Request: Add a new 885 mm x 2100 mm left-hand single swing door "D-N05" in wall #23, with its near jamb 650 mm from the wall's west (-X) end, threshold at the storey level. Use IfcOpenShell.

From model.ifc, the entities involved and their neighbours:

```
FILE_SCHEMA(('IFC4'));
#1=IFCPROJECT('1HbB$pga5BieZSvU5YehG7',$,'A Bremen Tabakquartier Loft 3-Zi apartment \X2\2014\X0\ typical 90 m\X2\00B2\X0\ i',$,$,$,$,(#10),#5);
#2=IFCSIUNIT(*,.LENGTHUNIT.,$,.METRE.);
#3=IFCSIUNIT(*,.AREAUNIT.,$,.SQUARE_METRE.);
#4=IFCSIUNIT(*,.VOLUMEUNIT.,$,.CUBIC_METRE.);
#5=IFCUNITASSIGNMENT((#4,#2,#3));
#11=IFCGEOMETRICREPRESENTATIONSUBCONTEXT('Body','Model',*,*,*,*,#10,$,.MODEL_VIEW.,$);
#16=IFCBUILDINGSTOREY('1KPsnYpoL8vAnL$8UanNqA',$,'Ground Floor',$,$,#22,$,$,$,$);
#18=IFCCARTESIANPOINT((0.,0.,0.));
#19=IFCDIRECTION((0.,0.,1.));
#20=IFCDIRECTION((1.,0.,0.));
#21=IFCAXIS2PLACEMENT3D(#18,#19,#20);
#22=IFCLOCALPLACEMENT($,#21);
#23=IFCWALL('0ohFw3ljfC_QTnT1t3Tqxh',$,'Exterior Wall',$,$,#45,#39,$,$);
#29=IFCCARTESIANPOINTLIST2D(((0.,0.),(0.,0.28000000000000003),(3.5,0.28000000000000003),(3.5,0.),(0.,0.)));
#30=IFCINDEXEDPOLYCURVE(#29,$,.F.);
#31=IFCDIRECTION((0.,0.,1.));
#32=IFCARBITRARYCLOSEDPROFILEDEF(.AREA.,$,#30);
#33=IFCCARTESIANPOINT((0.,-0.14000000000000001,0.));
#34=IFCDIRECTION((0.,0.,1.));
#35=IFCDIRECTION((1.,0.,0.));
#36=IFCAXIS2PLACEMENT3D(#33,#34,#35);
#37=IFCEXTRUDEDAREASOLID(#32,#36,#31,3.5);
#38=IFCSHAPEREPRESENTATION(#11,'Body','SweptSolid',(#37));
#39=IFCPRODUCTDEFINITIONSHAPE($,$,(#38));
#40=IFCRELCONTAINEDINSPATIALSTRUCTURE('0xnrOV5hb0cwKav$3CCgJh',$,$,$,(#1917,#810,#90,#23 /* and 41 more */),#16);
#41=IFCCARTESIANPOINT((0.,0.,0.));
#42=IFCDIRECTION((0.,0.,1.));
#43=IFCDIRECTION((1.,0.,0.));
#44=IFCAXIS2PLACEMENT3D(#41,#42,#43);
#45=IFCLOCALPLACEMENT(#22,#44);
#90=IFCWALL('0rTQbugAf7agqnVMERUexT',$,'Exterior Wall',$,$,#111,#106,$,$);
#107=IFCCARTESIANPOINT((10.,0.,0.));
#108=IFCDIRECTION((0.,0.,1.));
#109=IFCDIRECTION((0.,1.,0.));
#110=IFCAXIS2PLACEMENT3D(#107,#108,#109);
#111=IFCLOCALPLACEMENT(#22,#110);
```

```python
import numpy as np
import ifcopenshell
import ifcopenshell.api.feature
import ifcopenshell.api.geometry
import ifcopenshell.api.root
import ifcopenshell.api.spatial
import ifcopenshell.geom
import ifcopenshell.util.element
import ifcopenshell.util.placement
import ifcopenshell.util.representation
import ifcopenshell.util.shape
import ifcopenshell.util.unit

model = ifcopenshell.open("model.ifc")
unit_scale = ifcopenshell.util.unit.calculate_unit_scale(model)
settings = ifcopenshell.geom.settings()


def volume(element):
    """Net volume in cubic metres, openings subtracted."""
    shape = ifcopenshell.geom.create_shape(settings, element)
    return ifcopenshell.util.shape.get_volume(shape.geometry)


wall = model.by_guid("0ohFw3ljfC_QTnT1t3Tqxh")
storey = ifcopenshell.util.element.get_container(wall, ifc_class="IfcBuildingStorey")
context = ifcopenshell.util.representation.get_context(model, "Model", "Body", "MODEL_VIEW")
before = volume(wall)

width, height, from_end, sill = 0.885, 2.1, 0.65, 0.0  # metres

# The wall runs along its own X axis, and the end named is its -X end.
wall_shape = ifcopenshell.geom.create_shape(settings, wall)
x, y, z = ifcopenshell.util.shape.get_vertices(wall_shape.geometry).T
start = x.min() + from_end
face, thickness = float(y.min()), float(y.max() - y.min())
wall_matrix = ifcopenshell.util.placement.get_local_placement(wall.ObjectPlacement)
level = ifcopenshell.util.placement.get_local_placement(storey.ObjectPlacement)[2, 3]


def in_wall(x, y):
    """Placement at x, y metres in the wall's axes, at sill height."""
    matrix = wall_matrix.copy()
    matrix[:, 3] = wall_matrix @ np.array([x / unit_scale, y / unit_scale, 0.0, 1.0])
    matrix[2, 3] = level + sill / unit_scale
    return matrix


# Opening: a box that overshoots both wall faces by 50 mm.
opening = ifcopenshell.api.root.create_entity(model, ifc_class="IfcOpeningElement", predefined_type="OPENING")
box = ifcopenshell.api.geometry.add_wall_representation(
    model, context=context, length=width, height=height, thickness=thickness + 0.1
)
ifcopenshell.api.geometry.assign_representation(model, product=opening, representation=box)
ifcopenshell.api.geometry.edit_object_placement(model, product=opening, matrix=in_wall(start, face - 0.05), is_si=False)
ifcopenshell.api.feature.add_feature(model, feature=opening, element=wall)

door = ifcopenshell.api.root.create_entity(model, ifc_class="IfcDoor", name="D-N05", predefined_type="DOOR")
door.OverallWidth, door.OverallHeight = width / unit_scale, height / unit_scale
door.OperationType = "SINGLE_SWING_LEFT"
body = ifcopenshell.api.geometry.add_door_representation(
    model,
    context=context,
    overall_width=door.OverallWidth,
    overall_height=door.OverallHeight,
    operation_type="SINGLE_SWING_LEFT",
    lining_properties={"LiningDepth": thickness / unit_scale, "ThresholdDepth": thickness / unit_scale},
)
ifcopenshell.api.geometry.assign_representation(model, product=door, representation=body)
ifcopenshell.api.spatial.assign_container(model, products=[door], relating_structure=storey)
ifcopenshell.api.feature.add_filling(model, opening=opening, element=door)

# The lining spans the wall, so the door starts at the wall face.
ifcopenshell.api.geometry.edit_object_placement(model, product=door, matrix=in_wall(start, face), is_si=False)

after = volume(wall)

print(f"wall volume {before:.3f} -> {after:.3f} m3")

model.write("model_rev.ifc")
```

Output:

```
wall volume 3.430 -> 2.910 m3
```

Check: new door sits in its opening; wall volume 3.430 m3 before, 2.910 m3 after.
